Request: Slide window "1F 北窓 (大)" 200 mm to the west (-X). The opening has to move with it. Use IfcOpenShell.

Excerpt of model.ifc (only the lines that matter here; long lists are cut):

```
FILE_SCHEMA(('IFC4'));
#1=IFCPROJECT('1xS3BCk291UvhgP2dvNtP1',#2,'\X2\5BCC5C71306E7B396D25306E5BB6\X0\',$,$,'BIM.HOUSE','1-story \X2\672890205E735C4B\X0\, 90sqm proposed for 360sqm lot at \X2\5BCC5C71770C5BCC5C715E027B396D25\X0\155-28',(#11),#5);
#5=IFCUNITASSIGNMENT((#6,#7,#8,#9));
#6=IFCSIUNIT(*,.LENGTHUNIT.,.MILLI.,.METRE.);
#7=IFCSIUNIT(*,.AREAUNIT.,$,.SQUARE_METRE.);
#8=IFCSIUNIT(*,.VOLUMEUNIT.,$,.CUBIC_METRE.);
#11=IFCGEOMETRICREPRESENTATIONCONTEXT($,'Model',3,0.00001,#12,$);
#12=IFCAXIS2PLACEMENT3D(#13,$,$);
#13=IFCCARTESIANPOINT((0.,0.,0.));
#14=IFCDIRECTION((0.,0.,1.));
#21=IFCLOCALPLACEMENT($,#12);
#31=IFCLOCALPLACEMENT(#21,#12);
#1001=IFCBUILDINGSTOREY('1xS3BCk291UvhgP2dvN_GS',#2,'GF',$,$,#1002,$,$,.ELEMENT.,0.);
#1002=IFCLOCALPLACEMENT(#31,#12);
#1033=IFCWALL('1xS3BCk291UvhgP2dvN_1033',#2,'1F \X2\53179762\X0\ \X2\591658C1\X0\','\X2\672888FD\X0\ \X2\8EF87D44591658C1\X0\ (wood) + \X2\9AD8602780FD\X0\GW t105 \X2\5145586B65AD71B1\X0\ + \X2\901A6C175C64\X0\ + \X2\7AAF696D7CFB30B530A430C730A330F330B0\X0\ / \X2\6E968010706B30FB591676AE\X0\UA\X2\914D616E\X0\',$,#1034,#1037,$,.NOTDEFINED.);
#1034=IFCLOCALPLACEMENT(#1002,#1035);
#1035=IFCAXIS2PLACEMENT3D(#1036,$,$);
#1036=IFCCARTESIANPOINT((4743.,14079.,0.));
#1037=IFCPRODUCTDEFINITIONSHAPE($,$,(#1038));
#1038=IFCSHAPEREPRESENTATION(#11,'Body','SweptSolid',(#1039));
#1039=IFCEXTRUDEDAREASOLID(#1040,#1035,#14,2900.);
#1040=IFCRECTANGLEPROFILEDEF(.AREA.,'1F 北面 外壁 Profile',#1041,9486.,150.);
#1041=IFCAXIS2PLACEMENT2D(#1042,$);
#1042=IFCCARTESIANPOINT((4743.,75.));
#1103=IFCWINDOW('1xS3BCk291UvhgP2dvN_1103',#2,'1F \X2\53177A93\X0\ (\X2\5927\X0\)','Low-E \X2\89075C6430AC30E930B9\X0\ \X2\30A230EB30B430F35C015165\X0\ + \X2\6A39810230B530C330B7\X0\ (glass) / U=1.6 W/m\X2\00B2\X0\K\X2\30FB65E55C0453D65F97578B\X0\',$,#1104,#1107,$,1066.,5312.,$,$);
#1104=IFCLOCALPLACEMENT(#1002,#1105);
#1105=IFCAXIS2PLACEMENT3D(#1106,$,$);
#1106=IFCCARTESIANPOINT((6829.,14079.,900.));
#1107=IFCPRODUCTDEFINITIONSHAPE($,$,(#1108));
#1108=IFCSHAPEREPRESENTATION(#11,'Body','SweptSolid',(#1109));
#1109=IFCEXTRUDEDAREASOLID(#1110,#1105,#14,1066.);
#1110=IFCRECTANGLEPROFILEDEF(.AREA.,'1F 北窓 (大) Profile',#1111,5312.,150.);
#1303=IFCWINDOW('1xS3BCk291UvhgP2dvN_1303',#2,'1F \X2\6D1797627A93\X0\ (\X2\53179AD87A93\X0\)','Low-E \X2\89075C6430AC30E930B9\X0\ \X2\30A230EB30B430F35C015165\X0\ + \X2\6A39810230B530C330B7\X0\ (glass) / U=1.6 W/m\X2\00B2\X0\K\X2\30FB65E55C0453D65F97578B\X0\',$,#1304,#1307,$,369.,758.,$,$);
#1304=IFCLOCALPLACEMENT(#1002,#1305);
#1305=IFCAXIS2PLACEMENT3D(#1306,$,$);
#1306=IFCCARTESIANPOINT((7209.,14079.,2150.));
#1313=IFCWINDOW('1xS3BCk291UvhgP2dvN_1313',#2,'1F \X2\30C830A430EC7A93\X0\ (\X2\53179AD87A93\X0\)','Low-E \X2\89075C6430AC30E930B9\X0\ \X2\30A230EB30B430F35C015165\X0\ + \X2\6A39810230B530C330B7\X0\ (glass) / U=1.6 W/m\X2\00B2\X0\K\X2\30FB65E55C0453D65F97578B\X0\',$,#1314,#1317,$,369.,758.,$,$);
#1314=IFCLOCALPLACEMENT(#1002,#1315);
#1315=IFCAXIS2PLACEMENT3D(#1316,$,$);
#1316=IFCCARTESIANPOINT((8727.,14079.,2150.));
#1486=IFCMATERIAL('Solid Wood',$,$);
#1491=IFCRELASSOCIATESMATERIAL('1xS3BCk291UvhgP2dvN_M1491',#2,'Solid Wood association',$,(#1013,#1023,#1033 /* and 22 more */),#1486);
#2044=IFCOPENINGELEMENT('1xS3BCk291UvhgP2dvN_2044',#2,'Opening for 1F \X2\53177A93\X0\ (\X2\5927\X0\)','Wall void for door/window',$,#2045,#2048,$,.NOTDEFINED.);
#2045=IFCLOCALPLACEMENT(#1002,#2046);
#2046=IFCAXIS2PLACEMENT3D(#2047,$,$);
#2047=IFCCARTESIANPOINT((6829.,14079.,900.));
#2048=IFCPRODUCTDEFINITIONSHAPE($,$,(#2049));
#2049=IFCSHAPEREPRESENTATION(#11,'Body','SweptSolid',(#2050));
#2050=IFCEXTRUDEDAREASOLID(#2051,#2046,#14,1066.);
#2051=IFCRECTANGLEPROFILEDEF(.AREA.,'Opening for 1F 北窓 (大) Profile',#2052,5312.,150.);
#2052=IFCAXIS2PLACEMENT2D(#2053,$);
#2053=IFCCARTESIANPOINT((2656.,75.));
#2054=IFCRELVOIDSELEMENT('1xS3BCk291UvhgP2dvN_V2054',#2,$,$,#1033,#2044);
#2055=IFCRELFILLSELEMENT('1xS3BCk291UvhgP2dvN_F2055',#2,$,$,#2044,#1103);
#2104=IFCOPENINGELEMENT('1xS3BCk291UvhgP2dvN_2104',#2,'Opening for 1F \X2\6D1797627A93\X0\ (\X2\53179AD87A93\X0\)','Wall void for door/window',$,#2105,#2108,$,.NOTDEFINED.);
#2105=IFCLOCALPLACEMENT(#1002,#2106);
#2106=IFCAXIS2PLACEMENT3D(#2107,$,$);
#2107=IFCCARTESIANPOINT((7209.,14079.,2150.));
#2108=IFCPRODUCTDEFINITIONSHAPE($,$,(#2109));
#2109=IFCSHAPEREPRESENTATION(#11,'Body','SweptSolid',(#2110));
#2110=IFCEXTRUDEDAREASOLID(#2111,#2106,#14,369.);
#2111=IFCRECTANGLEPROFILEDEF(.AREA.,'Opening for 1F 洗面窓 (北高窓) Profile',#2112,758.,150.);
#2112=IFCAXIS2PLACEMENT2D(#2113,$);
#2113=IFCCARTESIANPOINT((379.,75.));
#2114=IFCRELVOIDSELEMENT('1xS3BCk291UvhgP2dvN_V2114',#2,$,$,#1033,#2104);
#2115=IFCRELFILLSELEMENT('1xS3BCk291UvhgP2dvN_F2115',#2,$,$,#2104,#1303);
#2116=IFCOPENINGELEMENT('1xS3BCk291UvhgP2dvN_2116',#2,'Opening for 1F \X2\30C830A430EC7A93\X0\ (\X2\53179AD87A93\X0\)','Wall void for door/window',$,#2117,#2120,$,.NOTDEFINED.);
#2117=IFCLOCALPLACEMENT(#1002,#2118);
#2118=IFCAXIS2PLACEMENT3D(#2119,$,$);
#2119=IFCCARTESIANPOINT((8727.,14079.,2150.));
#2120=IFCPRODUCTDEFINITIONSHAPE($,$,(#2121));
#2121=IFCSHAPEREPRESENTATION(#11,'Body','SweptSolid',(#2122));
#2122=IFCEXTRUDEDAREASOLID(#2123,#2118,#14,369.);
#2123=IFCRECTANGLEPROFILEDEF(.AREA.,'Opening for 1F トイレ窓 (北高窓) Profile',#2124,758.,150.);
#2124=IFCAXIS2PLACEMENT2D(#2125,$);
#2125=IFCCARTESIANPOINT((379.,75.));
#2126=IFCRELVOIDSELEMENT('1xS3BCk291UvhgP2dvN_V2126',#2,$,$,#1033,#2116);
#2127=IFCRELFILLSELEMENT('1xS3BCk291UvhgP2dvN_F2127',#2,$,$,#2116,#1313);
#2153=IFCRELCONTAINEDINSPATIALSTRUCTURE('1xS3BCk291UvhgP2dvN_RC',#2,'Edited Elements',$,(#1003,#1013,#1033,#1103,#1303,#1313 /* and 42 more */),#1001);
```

```python
import ifcopenshell
import ifcopenshell.api.geometry
import ifcopenshell.util.placement
import ifcopenshell.util.unit

model = ifcopenshell.open("model.ifc")
unit_scale = ifcopenshell.util.unit.calculate_unit_scale(model)

window = model.by_guid("1xS3BCk291UvhgP2dvN_1103")
opening = window.FillsVoids[0].RelatingOpeningElement
wall = opening.VoidsElements[0].RelatingBuildingElement

wall_matrix = ifcopenshell.util.placement.get_local_placement(wall.ObjectPlacement)
shift = wall_matrix[:3, 0] * -0.2 / unit_scale
before = ifcopenshell.util.placement.get_local_placement(window.ObjectPlacement)[:3, 3].copy()

# The window is not placed relative to its opening, so move both.
for product in (opening, window):
    matrix = ifcopenshell.util.placement.get_local_placement(product.ObjectPlacement)
    matrix[:3, 3] += shift
    ifcopenshell.api.geometry.edit_object_placement(model, product=product, matrix=matrix, is_si=False)

after = ifcopenshell.util.placement.get_local_placement(window.ObjectPlacement)[:3, 3]
print("window moved by", (after - before).round(3) + 0.0)

model.write("model_edited.ifc")
```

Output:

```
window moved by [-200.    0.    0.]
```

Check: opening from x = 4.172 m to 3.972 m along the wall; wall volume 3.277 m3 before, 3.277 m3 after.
